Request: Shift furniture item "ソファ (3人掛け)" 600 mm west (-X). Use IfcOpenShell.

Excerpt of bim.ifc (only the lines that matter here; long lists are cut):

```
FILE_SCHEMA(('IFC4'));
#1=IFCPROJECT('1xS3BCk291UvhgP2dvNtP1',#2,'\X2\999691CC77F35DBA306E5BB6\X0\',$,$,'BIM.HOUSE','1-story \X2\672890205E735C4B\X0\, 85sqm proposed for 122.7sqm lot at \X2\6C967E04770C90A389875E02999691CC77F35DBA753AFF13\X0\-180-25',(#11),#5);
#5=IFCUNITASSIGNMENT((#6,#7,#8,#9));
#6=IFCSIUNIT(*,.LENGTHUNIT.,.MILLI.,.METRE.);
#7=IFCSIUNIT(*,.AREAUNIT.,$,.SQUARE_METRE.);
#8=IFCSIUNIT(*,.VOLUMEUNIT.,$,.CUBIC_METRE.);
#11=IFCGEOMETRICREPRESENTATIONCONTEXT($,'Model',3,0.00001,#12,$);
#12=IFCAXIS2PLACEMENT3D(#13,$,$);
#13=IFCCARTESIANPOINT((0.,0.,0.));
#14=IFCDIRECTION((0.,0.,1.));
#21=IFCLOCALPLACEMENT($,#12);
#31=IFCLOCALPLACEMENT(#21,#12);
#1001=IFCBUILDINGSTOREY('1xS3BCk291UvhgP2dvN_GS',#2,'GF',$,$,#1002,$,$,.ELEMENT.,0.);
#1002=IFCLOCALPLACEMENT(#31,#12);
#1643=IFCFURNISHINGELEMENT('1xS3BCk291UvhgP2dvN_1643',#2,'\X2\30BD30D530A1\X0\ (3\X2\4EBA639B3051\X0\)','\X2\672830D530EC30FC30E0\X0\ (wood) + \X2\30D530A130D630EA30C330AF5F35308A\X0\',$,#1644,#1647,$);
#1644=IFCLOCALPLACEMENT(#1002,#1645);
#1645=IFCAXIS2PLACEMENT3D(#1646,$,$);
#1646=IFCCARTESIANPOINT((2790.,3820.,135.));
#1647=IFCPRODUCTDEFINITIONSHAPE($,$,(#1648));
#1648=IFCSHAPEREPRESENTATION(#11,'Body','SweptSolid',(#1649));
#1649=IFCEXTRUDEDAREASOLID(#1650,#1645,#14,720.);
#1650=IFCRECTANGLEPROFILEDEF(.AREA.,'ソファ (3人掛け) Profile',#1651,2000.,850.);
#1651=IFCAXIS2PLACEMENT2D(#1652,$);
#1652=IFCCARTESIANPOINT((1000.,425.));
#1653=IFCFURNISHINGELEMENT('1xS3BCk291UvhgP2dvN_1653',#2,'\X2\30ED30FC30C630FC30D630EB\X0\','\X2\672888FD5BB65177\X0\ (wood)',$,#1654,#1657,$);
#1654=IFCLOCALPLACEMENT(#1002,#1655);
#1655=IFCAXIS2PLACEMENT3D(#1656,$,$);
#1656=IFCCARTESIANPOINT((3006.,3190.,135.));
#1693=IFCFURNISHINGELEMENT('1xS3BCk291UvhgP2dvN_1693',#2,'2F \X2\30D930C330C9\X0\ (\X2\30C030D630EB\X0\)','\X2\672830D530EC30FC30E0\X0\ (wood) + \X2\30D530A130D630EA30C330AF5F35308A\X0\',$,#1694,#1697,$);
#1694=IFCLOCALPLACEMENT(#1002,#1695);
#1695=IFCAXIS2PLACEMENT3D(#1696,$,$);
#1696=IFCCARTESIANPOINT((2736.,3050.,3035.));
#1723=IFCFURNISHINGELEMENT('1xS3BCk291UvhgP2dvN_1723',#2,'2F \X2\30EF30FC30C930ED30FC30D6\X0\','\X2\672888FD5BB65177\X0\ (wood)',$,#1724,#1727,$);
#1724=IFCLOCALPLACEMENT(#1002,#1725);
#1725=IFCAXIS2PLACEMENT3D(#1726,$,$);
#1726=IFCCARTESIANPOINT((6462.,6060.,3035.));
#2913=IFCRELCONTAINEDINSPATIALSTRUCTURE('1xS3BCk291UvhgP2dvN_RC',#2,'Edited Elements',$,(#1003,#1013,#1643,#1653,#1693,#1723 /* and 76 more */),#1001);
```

```python
import ifcopenshell
import ifcopenshell.api.geometry
import ifcopenshell.util.placement

model = ifcopenshell.open("bim.ifc")

item = model.by_guid("1xS3BCk291UvhgP2dvN_1643")
matrix = ifcopenshell.util.placement.get_local_placement(item.ObjectPlacement)
matrix[0, 3] -= 600.0
ifcopenshell.api.geometry.edit_object_placement(model, product=item, matrix=matrix, is_si=False)

print(ifcopenshell.util.placement.get_local_placement(item.ObjectPlacement).round(3) + 0.0)

model.write("bim_edited.ifc")
```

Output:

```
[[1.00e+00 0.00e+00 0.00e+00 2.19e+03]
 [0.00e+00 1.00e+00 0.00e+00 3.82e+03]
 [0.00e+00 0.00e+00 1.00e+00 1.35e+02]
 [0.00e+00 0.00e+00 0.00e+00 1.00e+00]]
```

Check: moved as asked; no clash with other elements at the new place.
